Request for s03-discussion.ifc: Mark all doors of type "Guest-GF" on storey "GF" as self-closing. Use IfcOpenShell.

First a look at what the model holds.

```python
import ifcopenshell
import ifcopenshell.util.element

model = ifcopenshell.open("s03-discussion.ifc")
print(model.schema)
storey = next(s for s in model.by_type("IfcBuildingStorey") if s.Name == "GF")
doors = [e for e in ifcopenshell.util.element.get_decomposition(storey) if e.is_a("IfcDoor")]
seen = {}
for e in doors:
    element_type = ifcopenshell.util.element.get_type(e)
    key = (element_type.Name if element_type != e and element_type else None, ifcopenshell.util.element.get_pset(e, "Pset_DoorCommon", "SelfClosing"))
    seen[key] = seen.get(key, 0) + 1
for (name, value), count in sorted(seen.items(), key=str):
    print(count, "x", name, "|", value)
```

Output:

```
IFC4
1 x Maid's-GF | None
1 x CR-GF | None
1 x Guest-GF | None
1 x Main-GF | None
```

```python
import ifcopenshell
import ifcopenshell.api.pset
import ifcopenshell.util.element

model = ifcopenshell.open("s03-discussion.ifc")

storey = next(s for s in model.by_type("IfcBuildingStorey") if s.Name == "GF")
doors = [e for e in ifcopenshell.util.element.get_decomposition(storey) if e.is_a("IfcDoor")]

count = 0
for e in doors:
    element_type = ifcopenshell.util.element.get_type(e)
    if element_type in (None, e) or element_type.Name != "Guest-GF":
        continue
    # add_pset returns the element's existing set when there is one.
    pset = ifcopenshell.api.pset.add_pset(model, product=e, name="Pset_DoorCommon")
    ifcopenshell.api.pset.edit_pset(model, pset=pset, properties={"SelfClosing": True})
    count += 1

print(count, "doors updated")

model.write("s03-discussion-out.ifc")
```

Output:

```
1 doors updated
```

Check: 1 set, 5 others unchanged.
